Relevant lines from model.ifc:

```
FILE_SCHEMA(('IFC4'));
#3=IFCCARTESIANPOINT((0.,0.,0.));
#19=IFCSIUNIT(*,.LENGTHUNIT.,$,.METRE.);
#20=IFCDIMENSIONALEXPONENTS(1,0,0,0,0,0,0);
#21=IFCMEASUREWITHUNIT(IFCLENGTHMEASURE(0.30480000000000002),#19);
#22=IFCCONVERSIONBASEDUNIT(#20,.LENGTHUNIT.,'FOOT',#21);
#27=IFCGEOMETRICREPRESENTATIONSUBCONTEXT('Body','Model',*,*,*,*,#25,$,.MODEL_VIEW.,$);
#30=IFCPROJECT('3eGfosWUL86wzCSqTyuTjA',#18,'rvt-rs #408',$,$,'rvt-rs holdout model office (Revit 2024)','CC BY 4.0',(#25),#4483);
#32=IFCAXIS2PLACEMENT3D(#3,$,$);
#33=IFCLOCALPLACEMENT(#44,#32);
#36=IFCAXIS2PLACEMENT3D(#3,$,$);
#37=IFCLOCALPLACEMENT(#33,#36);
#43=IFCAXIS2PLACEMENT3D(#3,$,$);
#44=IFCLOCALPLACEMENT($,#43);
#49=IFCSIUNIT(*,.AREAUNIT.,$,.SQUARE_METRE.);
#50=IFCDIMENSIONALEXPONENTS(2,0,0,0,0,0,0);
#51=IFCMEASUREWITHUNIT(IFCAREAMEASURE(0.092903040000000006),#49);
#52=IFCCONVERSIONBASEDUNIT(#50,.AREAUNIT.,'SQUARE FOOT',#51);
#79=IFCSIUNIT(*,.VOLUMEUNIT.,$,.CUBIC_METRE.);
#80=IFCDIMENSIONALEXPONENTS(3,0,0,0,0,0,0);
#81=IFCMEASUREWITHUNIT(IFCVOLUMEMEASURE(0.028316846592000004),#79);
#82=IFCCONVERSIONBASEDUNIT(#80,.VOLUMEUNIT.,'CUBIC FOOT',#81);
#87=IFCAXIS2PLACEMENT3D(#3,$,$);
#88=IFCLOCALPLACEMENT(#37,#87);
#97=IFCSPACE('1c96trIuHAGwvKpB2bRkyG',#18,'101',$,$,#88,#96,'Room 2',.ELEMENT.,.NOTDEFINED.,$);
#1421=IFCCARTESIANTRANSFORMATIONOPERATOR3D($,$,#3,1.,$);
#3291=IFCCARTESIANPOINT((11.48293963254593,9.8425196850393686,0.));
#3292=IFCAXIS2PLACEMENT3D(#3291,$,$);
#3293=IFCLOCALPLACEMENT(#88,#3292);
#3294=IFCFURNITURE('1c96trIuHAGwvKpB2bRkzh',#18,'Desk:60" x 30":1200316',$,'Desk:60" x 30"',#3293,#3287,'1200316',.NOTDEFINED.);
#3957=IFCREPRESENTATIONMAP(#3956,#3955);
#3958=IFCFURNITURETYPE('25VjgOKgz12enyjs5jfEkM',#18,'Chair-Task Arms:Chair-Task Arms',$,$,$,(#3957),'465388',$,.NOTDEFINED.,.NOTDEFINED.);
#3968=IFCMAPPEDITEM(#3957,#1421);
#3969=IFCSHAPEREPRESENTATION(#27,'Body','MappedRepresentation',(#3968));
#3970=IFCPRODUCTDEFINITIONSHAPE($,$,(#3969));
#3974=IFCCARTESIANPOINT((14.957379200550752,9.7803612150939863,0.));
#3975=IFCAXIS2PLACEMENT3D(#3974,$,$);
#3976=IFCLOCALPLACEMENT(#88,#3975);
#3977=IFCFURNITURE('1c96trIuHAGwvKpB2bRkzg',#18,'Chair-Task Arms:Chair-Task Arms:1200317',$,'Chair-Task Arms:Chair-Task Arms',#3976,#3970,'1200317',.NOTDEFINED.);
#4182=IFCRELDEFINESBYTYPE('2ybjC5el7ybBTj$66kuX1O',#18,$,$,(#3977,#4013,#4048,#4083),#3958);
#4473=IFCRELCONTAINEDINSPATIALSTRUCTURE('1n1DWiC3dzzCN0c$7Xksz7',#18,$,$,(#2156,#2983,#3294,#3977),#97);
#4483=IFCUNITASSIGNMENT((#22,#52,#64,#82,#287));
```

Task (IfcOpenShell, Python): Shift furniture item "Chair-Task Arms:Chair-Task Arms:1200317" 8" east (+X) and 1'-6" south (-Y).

```python
import ifcopenshell
import ifcopenshell.api.geometry
import ifcopenshell.util.placement
import ifcopenshell.util.unit

model = ifcopenshell.open("model.ifc")
unit_scale = ifcopenshell.util.unit.calculate_unit_scale(model)

item = model.by_guid("1c96trIuHAGwvKpB2bRkzg")
matrix = ifcopenshell.util.placement.get_local_placement(item.ObjectPlacement)
matrix[0, 3] += 8 * 0.0254 / unit_scale
matrix[1, 3] -= 18 * 0.0254 / unit_scale
ifcopenshell.api.geometry.edit_object_placement(model, product=item, matrix=matrix, is_si=False)

print(ifcopenshell.util.placement.get_local_placement(item.ObjectPlacement).round(3) + 0.0)

model.write("model-out.ifc")
```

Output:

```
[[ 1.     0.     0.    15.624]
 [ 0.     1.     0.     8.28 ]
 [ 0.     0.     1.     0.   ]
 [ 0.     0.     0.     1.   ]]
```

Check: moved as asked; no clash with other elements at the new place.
